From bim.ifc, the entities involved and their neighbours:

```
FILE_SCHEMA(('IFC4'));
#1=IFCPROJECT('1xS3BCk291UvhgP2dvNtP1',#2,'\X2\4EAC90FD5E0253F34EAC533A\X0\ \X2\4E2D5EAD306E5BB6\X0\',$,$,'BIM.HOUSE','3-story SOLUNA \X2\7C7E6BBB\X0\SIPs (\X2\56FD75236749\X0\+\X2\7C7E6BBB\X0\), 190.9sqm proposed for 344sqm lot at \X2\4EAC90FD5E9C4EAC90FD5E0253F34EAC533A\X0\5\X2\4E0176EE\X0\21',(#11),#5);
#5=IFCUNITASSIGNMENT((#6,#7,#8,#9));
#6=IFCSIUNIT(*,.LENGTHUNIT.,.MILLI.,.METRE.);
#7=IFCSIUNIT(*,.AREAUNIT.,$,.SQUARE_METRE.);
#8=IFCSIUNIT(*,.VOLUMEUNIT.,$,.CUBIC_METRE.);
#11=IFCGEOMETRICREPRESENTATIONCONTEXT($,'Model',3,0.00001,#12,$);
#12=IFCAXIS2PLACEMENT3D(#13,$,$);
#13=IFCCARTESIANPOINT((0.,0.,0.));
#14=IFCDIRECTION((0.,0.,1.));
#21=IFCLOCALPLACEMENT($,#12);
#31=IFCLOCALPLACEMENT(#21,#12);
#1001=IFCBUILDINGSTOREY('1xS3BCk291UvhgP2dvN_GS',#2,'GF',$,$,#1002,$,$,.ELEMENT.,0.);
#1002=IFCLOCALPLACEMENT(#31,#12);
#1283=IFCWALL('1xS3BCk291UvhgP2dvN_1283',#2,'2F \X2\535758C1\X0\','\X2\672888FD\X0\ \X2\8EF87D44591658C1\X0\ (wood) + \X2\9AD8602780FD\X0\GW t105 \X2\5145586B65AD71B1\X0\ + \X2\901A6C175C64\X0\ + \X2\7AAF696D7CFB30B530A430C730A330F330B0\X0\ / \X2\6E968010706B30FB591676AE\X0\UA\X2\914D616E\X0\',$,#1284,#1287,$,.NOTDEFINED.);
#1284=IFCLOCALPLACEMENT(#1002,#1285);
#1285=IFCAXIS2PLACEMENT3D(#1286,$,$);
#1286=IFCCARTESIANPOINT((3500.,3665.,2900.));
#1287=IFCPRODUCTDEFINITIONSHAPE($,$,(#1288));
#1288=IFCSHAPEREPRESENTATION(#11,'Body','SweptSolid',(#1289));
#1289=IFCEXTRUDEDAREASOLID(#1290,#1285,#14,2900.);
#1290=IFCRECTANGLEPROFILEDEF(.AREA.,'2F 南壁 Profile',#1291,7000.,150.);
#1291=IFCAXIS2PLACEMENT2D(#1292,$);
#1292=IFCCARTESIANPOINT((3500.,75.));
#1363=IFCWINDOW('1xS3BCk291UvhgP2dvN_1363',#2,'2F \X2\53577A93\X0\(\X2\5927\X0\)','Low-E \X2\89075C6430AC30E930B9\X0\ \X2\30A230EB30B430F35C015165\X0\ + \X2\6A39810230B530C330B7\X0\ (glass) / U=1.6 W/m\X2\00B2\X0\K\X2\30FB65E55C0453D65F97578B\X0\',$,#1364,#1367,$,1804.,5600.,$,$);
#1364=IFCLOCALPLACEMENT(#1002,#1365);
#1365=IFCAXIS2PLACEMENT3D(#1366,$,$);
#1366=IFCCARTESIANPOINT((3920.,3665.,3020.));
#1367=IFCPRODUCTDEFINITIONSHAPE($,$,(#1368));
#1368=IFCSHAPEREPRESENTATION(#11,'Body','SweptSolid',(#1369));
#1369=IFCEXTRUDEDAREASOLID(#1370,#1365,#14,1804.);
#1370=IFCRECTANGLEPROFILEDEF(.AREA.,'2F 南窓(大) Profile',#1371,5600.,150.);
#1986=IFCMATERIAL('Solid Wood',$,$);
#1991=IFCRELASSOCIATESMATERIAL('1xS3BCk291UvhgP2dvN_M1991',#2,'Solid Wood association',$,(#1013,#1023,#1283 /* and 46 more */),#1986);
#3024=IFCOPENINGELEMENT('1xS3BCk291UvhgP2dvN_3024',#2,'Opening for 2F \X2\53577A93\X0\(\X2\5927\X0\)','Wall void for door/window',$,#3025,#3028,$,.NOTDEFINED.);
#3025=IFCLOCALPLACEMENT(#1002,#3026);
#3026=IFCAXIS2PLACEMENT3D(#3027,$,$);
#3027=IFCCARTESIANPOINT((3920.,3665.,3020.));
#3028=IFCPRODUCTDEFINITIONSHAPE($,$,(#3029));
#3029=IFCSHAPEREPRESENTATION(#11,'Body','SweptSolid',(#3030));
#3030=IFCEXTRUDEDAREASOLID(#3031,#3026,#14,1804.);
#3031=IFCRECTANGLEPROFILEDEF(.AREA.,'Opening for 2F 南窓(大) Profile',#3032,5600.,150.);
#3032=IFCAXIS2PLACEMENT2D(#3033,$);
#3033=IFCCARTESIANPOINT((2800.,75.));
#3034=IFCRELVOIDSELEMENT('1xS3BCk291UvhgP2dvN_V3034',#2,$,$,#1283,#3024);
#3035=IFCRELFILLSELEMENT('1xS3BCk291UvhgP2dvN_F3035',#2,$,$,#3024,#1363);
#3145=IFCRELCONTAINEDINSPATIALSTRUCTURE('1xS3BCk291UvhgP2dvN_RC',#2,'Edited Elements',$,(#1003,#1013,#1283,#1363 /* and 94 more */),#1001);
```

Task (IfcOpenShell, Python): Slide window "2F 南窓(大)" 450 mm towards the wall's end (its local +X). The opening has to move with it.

```python
import ifcopenshell
import ifcopenshell.api.geometry
import ifcopenshell.util.placement
import ifcopenshell.util.unit

model = ifcopenshell.open("bim.ifc")
unit_scale = ifcopenshell.util.unit.calculate_unit_scale(model)

window = model.by_guid("1xS3BCk291UvhgP2dvN_1363")
opening = window.FillsVoids[0].RelatingOpeningElement
wall = opening.VoidsElements[0].RelatingBuildingElement

wall_matrix = ifcopenshell.util.placement.get_local_placement(wall.ObjectPlacement)
shift = wall_matrix[:3, 0] * 0.45 / unit_scale
before = ifcopenshell.util.placement.get_local_placement(window.ObjectPlacement)[:3, 3].copy()

# The window is not placed relative to its opening, so move both.
for product in (opening, window):
    matrix = ifcopenshell.util.placement.get_local_placement(product.ObjectPlacement)
    matrix[:3, 3] += shift
    ifcopenshell.api.geometry.edit_object_placement(model, product=product, matrix=matrix, is_si=False)

after = ifcopenshell.util.placement.get_local_placement(window.ObjectPlacement)[:3, 3]
print("window moved by", (after - before).round(3) + 0.0)

model.write("bim_edited.ifc")
```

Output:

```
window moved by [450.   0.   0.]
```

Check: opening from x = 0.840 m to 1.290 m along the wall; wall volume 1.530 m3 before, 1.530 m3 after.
